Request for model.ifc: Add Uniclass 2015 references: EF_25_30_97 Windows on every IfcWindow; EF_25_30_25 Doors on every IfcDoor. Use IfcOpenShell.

First a look at what the model holds.

```python
import ifcopenshell

model = ifcopenshell.open("model.ifc")
print(model.schema)
print("classifications:", [c.Name for c in model.by_type("IfcClassification")])
for ifc_class in ("IfcDoor", "IfcRoof", "IfcStair", "IfcWall", "IfcWindow"):
    print(ifc_class, len(model.by_type(ifc_class)))
```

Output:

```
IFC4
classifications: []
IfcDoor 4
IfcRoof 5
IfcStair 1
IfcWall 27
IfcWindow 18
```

```python
import ifcopenshell
import ifcopenshell.api.classification

model = ifcopenshell.open("model.ifc")

system = ifcopenshell.api.classification.add_classification(model, classification="Uniclass 2015")

codes = {
    "IfcWindow": ("EF_25_30_97", "Windows"),
    "IfcDoor": ("EF_25_30_25", "Doors"),
}
for ifc_class, (code, name) in codes.items():
    products = model.by_type(ifc_class)
    ifcopenshell.api.classification.add_reference(
        model, products=products, classification=system, identification=code, name=name
    )
    print(code, len(products))

model.write("model_edited.ifc")
```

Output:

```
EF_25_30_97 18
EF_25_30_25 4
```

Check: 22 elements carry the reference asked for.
